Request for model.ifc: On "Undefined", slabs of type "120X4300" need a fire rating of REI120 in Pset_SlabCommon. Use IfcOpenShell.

First a look at what the model holds.

```python
import ifcopenshell
import ifcopenshell.util.element

model = ifcopenshell.open("model.ifc")
print(model.schema)
storey = next(s for s in model.by_type("IfcBuildingStorey") if s.Name == "Undefined")
slabs = [e for e in ifcopenshell.util.element.get_decomposition(storey) if e.is_a("IfcSlab")]
seen = {}
for e in slabs:
    element_type = ifcopenshell.util.element.get_type(e)
    key = (element_type.Name if element_type != e and element_type else None, ifcopenshell.util.element.get_pset(e, "Pset_SlabCommon", "FireRating"))
    seen[key] = seen.get(key, 0) + 1
for (name, value), count in sorted(seen.items(), key=str):
    print(count, "x", name, "|", value)
```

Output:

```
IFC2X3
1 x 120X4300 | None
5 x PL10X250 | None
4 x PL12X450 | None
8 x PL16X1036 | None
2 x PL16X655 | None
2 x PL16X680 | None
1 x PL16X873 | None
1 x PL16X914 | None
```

```python
import ifcopenshell
import ifcopenshell.api.pset
import ifcopenshell.util.element

model = ifcopenshell.open("model.ifc")

storey = next(s for s in model.by_type("IfcBuildingStorey") if s.Name == "Undefined")
slabs = [e for e in ifcopenshell.util.element.get_decomposition(storey) if e.is_a("IfcSlab")]

count = 0
for e in slabs:
    element_type = ifcopenshell.util.element.get_type(e)
    if element_type in (None, e) or element_type.Name != "120X4300":
        continue
    # add_pset returns the element's existing set when there is one.
    pset = ifcopenshell.api.pset.add_pset(model, product=e, name="Pset_SlabCommon")
    ifcopenshell.api.pset.edit_pset(model, pset=pset, properties={"FireRating": "REI120"})
    count += 1

print(count, "slabs updated")

model.write("model_rev.ifc")
```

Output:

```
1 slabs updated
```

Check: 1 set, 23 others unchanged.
